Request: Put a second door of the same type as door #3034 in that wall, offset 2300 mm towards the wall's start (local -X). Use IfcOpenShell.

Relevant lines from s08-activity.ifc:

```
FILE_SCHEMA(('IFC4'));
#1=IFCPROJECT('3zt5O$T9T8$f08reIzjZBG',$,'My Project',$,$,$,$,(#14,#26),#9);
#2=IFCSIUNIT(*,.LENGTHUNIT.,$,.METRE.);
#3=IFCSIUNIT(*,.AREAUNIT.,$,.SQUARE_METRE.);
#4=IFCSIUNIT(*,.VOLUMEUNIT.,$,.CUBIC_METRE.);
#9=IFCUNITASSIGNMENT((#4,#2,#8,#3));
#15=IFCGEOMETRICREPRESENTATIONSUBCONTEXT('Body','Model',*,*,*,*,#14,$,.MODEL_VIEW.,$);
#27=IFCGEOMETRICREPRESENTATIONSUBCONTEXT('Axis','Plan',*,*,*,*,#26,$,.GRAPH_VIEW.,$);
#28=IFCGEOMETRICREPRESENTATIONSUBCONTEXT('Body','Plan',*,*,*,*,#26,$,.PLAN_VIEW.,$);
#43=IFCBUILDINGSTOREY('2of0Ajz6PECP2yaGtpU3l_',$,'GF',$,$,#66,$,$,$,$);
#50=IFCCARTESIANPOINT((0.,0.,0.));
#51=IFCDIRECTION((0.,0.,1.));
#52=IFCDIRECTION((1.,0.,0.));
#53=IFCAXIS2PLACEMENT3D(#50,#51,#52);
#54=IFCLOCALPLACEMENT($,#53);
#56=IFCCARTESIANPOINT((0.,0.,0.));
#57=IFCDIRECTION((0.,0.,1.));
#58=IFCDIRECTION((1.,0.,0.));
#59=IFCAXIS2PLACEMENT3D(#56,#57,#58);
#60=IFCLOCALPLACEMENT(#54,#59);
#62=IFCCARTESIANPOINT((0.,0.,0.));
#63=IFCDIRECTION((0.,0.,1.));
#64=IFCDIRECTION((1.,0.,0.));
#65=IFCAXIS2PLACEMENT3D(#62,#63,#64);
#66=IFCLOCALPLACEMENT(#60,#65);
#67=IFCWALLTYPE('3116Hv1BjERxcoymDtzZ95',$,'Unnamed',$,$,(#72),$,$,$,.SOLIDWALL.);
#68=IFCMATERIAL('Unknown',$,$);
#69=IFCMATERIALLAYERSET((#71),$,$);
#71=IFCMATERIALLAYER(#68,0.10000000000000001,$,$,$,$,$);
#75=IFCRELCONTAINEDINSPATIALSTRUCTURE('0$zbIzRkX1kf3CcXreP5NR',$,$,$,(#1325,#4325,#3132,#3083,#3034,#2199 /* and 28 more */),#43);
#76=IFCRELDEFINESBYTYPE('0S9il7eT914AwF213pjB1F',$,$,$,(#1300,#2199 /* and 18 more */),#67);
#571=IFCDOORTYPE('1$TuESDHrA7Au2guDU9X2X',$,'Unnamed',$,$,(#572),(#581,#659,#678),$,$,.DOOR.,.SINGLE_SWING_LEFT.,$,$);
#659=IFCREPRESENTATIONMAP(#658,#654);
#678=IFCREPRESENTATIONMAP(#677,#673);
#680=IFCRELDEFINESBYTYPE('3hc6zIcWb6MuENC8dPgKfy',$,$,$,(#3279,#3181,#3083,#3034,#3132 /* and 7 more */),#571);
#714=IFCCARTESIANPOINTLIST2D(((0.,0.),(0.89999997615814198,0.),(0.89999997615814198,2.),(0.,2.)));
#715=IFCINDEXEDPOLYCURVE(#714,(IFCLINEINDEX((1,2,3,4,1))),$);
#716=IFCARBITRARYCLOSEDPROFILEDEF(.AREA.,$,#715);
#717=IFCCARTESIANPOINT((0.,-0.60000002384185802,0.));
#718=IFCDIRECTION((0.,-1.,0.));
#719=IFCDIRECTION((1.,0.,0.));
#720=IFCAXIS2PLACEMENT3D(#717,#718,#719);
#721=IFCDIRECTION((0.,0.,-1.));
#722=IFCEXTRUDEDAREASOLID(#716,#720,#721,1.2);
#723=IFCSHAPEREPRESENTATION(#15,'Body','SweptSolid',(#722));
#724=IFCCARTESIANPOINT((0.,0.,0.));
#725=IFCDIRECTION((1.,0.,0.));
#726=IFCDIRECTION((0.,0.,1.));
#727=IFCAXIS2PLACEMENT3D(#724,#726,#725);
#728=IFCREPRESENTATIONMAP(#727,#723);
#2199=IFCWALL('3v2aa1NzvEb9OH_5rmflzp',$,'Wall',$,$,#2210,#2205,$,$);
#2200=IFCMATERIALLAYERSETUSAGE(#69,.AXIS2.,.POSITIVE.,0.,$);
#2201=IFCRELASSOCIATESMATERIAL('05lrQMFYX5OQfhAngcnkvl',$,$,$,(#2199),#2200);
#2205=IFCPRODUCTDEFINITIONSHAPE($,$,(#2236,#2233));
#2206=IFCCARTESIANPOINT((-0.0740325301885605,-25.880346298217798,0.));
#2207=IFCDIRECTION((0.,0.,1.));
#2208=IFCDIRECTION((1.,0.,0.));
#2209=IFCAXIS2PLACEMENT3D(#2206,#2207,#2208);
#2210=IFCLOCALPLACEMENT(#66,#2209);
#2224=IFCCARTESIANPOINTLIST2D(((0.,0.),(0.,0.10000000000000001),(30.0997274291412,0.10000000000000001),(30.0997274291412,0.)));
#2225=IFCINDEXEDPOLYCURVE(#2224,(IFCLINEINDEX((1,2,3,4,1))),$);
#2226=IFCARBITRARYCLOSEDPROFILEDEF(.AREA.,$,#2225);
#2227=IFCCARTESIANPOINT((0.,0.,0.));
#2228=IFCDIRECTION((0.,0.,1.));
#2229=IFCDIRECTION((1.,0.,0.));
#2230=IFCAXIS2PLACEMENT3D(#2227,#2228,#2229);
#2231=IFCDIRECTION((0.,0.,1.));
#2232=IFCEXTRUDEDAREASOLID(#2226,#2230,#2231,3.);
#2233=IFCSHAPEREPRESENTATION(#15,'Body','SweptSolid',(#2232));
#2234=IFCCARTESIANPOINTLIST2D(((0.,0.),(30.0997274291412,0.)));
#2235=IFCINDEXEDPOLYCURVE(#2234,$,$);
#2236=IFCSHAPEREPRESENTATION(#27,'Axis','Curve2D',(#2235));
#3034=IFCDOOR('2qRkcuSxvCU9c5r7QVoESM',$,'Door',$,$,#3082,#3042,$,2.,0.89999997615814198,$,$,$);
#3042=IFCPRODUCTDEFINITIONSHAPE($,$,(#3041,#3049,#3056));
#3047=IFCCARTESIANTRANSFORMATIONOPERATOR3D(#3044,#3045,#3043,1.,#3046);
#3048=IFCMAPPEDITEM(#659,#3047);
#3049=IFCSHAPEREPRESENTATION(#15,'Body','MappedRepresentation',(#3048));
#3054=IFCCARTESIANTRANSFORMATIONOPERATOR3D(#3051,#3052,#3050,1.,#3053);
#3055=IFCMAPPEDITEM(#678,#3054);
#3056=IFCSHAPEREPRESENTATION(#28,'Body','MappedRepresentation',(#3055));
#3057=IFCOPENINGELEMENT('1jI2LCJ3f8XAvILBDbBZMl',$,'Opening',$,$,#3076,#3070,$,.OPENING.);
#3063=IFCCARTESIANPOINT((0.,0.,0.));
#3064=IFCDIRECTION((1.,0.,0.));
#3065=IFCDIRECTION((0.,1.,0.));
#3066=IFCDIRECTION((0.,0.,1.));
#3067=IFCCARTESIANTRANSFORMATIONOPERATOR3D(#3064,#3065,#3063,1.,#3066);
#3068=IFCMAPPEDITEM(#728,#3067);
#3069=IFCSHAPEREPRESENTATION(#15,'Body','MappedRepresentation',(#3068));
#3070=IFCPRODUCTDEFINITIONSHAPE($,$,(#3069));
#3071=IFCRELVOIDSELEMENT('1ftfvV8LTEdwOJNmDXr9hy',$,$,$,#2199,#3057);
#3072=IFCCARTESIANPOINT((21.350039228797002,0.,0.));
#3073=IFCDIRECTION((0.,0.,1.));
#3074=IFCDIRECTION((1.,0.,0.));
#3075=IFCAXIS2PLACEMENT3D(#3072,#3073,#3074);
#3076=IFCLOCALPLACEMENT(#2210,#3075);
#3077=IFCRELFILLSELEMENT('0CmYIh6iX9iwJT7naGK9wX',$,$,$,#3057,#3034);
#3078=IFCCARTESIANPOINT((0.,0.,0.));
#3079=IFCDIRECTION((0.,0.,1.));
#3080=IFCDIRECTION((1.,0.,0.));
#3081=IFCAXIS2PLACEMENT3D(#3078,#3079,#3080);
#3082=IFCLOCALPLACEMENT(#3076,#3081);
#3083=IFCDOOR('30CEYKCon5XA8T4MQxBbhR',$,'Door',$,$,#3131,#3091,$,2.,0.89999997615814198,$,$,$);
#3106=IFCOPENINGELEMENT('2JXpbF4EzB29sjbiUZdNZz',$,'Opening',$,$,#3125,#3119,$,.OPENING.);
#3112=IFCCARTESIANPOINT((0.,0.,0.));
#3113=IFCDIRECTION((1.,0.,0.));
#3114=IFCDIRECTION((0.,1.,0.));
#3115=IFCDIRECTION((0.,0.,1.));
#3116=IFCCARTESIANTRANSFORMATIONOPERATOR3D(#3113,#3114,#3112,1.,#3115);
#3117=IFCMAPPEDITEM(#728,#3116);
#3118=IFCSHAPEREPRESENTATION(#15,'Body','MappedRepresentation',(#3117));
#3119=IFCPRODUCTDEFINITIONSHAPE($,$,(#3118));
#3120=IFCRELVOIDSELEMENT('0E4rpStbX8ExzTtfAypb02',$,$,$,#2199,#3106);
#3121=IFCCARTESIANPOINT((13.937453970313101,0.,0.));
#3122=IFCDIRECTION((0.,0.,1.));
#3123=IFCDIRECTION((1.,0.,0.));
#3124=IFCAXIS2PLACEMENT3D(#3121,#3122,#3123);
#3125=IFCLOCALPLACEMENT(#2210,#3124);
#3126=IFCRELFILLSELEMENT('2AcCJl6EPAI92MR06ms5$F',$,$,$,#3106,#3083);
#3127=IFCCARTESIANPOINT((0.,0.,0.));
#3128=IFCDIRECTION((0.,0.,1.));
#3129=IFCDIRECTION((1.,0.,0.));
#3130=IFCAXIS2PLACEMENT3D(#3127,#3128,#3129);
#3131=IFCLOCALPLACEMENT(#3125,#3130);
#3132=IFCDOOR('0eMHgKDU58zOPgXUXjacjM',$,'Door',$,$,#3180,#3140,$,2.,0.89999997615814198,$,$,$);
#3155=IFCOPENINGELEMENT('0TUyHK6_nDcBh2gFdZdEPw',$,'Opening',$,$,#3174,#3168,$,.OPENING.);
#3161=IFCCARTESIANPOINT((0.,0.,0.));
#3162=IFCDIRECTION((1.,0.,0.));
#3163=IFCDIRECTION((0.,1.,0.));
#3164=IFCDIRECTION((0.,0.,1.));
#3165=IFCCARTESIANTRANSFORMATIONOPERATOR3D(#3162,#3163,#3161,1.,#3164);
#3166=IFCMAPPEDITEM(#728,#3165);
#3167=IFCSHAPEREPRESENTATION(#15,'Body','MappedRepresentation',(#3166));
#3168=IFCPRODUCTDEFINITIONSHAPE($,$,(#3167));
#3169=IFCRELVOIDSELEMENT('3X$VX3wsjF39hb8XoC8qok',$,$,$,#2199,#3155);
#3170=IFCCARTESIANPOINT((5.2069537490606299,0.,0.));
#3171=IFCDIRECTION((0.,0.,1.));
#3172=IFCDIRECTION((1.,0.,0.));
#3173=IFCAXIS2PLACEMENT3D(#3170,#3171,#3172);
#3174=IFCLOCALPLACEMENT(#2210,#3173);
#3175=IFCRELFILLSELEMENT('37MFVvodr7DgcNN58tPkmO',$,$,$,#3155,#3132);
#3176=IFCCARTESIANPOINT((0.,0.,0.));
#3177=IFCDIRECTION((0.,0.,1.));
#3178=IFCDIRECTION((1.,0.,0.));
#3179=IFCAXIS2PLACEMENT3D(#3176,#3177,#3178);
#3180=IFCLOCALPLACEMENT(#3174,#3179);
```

```python
import ifcopenshell
import ifcopenshell.api.feature
import ifcopenshell.api.geometry
import ifcopenshell.api.root
import ifcopenshell.geom
import ifcopenshell.util.element
import ifcopenshell.util.placement
import ifcopenshell.util.shape

model = ifcopenshell.open("s08-activity.ifc")
settings = ifcopenshell.geom.settings()


def volume(element):
    """Net volume in cubic metres, openings subtracted."""
    shape = ifcopenshell.geom.create_shape(settings, element)
    return ifcopenshell.util.shape.get_volume(shape.geometry)


door = model.by_guid("2qRkcuSxvCU9c5r7QVoESM")
opening = door.FillsVoids[0].RelatingOpeningElement
wall = opening.VoidsElements[0].RelatingBuildingElement
before = volume(wall)
shift = ifcopenshell.util.placement.get_local_placement(wall.ObjectPlacement)[:3, 0] * -2.3

# copy_class copies the void relationship, type, container and properties, but no geometry.
new_opening = ifcopenshell.api.root.copy_class(model, product=opening)
new_opening.Representation = ifcopenshell.util.element.copy_deep(
    model, opening.Representation, exclude=["IfcGeometricRepresentationContext", "IfcRepresentationMap"]
)
new_door = ifcopenshell.api.root.copy_class(model, product=door)
new_door.Representation = ifcopenshell.util.element.copy_deep(
    model, door.Representation, exclude=["IfcGeometricRepresentationContext", "IfcRepresentationMap"]
)
ifcopenshell.api.feature.add_filling(model, opening=new_opening, element=new_door)

for old, new in ((opening, new_opening), (door, new_door)):
    matrix = ifcopenshell.util.placement.get_local_placement(old.ObjectPlacement)
    matrix[:3, 3] += shift
    ifcopenshell.api.geometry.edit_object_placement(model, product=new, matrix=matrix, is_si=False)

after = volume(wall)

print(f"wall volume {before:.3f} -> {after:.3f} m3")

model.write("s08-activity_updated.ifc")
```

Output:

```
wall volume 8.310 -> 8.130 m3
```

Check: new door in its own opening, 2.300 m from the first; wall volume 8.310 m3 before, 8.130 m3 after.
